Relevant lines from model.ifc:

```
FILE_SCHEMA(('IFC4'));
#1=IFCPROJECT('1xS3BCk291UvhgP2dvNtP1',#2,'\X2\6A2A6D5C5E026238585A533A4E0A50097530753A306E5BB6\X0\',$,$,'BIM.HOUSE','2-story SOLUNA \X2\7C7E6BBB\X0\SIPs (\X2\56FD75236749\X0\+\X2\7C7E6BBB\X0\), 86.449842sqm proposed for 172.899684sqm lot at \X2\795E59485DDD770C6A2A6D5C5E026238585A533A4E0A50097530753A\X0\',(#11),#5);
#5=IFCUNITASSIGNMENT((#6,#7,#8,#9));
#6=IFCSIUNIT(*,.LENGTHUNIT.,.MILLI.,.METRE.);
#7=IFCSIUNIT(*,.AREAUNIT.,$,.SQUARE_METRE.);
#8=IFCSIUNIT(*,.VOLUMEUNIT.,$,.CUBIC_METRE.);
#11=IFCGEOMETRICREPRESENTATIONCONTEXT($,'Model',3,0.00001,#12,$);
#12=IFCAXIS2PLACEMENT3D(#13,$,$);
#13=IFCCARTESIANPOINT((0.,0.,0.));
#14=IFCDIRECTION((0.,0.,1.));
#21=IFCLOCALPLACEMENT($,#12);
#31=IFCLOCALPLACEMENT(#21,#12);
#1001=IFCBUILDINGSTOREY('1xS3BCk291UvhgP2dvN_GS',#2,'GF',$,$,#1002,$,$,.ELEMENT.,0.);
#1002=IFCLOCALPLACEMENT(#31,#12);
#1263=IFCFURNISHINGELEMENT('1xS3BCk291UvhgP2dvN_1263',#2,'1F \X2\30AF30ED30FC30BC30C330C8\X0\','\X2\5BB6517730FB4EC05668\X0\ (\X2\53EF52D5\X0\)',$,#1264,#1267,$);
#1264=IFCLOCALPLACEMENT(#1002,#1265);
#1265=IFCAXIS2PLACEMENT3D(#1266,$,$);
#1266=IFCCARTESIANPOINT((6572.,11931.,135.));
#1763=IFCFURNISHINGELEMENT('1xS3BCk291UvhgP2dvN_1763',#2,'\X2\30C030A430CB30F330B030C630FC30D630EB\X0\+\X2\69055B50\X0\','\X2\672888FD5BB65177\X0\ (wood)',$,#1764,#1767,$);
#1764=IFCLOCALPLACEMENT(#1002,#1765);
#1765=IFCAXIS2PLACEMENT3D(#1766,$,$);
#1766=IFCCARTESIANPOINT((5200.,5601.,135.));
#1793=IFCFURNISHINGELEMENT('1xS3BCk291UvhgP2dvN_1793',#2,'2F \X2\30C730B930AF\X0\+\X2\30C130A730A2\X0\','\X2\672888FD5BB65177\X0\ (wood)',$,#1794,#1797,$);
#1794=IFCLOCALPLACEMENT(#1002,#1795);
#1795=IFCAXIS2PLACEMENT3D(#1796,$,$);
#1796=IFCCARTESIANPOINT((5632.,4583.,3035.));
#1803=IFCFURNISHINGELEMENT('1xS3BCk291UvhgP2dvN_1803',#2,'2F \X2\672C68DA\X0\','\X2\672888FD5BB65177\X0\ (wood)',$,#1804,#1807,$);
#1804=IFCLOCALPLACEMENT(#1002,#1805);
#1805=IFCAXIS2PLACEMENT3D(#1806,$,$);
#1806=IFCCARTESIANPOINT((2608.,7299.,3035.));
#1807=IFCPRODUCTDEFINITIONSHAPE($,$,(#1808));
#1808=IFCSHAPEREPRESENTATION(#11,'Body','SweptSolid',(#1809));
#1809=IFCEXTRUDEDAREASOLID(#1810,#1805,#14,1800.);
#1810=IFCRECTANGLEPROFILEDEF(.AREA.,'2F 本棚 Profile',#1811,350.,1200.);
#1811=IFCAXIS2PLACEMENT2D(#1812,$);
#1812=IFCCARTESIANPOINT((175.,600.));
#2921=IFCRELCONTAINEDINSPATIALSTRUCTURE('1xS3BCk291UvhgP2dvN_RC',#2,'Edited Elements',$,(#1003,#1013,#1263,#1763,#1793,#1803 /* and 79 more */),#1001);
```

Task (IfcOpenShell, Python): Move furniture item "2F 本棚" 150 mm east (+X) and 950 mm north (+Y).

```python
import ifcopenshell
import ifcopenshell.api.geometry
import ifcopenshell.util.placement

model = ifcopenshell.open("model.ifc")

item = model.by_id(1803)
matrix = ifcopenshell.util.placement.get_local_placement(item.ObjectPlacement)
matrix[0, 3] += 150.0
matrix[1, 3] += 950.0
ifcopenshell.api.geometry.edit_object_placement(model, product=item, matrix=matrix, is_si=False)

print(ifcopenshell.util.placement.get_local_placement(item.ObjectPlacement).round(3) + 0.0)

model.write("model_updated.ifc")
```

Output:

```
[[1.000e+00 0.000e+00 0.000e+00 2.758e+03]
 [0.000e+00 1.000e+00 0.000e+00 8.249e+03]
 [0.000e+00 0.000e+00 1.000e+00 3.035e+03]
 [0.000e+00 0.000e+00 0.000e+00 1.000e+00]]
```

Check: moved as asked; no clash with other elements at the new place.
